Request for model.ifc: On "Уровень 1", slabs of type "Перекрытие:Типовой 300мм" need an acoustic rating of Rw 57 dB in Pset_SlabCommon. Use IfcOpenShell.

First a look at what the model holds.

```python
import ifcopenshell
import ifcopenshell.util.element

model = ifcopenshell.open("model.ifc")
print(model.schema)
storey = next(s for s in model.by_type("IfcBuildingStorey") if s.Name == "Уровень 1")
slabs = [e for e in ifcopenshell.util.element.get_decomposition(storey) if e.is_a("IfcSlab")]
seen = {}
for e in slabs:
    element_type = ifcopenshell.util.element.get_type(e)
    key = (element_type.Name if element_type != e and element_type else None, ifcopenshell.util.element.get_pset(e, "Pset_SlabCommon", "AcousticRating"))
    seen[key] = seen.get(key, 0) + 1
for (name, value), count in sorted(seen.items(), key=str):
    print(count, "x", name, "|", value)
```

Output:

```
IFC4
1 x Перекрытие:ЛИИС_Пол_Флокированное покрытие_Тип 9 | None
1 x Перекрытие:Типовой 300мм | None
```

```python
import ifcopenshell
import ifcopenshell.api.pset
import ifcopenshell.util.element

model = ifcopenshell.open("model.ifc")

storey = next(s for s in model.by_type("IfcBuildingStorey") if s.Name == "Уровень 1")
slabs = [e for e in ifcopenshell.util.element.get_decomposition(storey) if e.is_a("IfcSlab")]

count = 0
for e in slabs:
    element_type = ifcopenshell.util.element.get_type(e)
    if element_type in (None, e) or element_type.Name != "Перекрытие:Типовой 300мм":
        continue
    # add_pset returns the element's existing set when there is one.
    pset = ifcopenshell.api.pset.add_pset(model, product=e, name="Pset_SlabCommon")
    ifcopenshell.api.pset.edit_pset(model, pset=pset, properties={"AcousticRating": "Rw 57 dB"})
    count += 1

print(count, "slabs updated")

model.write("model_v2.ifc")
```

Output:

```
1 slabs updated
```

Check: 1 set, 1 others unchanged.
